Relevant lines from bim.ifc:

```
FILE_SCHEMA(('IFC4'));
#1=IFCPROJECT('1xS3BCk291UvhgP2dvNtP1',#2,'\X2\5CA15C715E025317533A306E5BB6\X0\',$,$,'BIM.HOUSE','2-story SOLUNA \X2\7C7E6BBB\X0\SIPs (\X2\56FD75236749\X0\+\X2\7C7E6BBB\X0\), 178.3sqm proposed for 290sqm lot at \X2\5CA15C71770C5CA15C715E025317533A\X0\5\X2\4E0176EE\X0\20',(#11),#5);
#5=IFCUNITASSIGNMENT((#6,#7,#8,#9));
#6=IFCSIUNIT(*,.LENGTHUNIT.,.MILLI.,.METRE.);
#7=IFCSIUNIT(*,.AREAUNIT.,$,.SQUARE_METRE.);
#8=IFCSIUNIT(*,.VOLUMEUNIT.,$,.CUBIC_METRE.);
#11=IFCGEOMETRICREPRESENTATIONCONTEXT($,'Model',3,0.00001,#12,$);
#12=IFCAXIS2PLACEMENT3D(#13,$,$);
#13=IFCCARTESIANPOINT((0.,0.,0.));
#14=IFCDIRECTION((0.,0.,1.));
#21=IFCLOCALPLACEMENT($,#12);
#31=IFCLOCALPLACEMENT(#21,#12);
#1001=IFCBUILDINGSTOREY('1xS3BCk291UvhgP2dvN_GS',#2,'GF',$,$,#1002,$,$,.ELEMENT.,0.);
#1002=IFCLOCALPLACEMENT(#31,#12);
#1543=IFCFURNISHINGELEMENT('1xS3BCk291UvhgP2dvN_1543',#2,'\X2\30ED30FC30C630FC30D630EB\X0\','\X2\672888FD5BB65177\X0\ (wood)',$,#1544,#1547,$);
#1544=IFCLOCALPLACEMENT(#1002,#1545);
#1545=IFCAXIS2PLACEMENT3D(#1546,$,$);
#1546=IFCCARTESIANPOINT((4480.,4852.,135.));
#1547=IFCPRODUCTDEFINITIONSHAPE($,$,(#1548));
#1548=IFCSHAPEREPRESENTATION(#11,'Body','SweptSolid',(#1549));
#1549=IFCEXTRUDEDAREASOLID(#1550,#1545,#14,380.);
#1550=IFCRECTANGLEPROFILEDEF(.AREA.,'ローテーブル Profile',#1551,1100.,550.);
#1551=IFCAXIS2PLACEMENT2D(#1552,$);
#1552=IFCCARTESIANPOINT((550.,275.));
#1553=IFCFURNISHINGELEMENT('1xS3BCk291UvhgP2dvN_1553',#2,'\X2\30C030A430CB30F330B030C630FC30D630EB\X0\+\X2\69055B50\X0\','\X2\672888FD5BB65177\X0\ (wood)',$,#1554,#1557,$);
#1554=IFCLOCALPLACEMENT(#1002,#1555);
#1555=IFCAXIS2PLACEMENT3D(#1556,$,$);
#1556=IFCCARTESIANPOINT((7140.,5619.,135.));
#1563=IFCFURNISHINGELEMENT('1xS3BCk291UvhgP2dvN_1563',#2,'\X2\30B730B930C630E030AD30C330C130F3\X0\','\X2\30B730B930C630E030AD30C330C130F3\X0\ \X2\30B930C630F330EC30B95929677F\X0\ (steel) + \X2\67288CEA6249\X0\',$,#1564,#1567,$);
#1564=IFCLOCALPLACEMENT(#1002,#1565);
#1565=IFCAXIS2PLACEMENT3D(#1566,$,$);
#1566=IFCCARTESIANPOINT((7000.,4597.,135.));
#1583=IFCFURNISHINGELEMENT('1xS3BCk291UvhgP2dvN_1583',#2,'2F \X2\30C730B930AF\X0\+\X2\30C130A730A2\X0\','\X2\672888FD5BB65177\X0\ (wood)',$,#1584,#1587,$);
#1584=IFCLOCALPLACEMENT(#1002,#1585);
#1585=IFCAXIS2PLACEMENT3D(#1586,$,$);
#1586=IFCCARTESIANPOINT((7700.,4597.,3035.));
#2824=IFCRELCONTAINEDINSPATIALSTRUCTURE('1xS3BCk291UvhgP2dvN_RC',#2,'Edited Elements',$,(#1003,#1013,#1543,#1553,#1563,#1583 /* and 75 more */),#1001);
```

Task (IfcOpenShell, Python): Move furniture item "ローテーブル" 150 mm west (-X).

```python
import ifcopenshell
import ifcopenshell.api.geometry
import ifcopenshell.util.placement
import ifcopenshell.util.unit

model = ifcopenshell.open("bim.ifc")
unit_scale = ifcopenshell.util.unit.calculate_unit_scale(model)

item = model.by_guid("1xS3BCk291UvhgP2dvN_1543")
matrix = ifcopenshell.util.placement.get_local_placement(item.ObjectPlacement)
matrix[0, 3] -= 0.15 / unit_scale
ifcopenshell.api.geometry.edit_object_placement(model, product=item, matrix=matrix, is_si=False)

print(ifcopenshell.util.placement.get_local_placement(item.ObjectPlacement).round(3) + 0.0)

model.write("bim_edited.ifc")
```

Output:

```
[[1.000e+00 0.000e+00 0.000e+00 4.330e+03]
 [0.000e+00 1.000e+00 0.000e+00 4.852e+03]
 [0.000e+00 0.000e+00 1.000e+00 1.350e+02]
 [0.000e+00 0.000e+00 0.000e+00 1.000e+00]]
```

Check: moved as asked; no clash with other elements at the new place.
